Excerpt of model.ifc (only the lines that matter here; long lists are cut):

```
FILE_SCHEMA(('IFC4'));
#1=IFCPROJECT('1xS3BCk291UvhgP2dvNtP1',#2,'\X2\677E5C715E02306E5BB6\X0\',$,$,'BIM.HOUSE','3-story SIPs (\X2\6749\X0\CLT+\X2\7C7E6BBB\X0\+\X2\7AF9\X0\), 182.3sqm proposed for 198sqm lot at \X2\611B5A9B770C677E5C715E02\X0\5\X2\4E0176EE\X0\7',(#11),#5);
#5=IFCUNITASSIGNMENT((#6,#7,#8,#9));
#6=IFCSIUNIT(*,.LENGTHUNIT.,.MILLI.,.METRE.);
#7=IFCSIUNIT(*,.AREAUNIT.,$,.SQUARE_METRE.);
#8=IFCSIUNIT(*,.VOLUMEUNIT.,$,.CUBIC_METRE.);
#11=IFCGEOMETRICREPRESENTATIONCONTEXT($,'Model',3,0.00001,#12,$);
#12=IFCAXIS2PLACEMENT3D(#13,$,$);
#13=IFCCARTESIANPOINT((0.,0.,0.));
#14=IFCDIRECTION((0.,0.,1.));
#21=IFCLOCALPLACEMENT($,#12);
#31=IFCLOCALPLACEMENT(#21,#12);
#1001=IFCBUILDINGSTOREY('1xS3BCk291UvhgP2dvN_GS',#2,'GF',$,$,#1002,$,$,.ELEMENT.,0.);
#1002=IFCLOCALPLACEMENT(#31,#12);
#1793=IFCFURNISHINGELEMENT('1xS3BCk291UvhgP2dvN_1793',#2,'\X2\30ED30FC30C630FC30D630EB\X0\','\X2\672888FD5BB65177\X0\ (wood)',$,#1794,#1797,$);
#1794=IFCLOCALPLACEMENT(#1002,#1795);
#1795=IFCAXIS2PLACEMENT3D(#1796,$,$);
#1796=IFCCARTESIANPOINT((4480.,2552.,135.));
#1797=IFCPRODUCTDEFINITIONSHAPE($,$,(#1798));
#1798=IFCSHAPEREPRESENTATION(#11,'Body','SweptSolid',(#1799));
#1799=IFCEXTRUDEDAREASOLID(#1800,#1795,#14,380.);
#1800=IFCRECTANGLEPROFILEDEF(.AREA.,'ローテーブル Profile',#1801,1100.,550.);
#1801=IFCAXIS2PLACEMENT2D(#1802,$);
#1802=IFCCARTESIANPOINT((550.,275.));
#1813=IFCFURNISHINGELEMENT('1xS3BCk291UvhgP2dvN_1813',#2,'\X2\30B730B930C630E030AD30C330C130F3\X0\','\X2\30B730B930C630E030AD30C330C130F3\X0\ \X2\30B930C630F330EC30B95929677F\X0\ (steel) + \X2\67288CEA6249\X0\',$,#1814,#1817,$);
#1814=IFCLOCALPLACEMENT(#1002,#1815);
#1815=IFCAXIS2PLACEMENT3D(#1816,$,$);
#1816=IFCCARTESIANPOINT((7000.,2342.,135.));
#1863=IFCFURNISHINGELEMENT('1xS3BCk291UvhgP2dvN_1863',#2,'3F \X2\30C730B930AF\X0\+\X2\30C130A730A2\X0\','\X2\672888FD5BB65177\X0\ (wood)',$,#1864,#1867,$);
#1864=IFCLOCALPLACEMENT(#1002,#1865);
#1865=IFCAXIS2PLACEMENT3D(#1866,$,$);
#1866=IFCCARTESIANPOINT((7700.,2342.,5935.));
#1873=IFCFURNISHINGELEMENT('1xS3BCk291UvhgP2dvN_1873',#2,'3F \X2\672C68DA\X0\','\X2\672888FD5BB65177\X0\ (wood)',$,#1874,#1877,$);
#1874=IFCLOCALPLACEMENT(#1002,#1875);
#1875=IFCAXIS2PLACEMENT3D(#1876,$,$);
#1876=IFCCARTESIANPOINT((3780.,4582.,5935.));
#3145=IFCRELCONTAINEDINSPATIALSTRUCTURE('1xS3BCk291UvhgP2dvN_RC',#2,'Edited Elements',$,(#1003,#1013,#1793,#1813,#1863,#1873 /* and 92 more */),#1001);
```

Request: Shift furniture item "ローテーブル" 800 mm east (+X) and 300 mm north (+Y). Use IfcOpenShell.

```python
import ifcopenshell
import ifcopenshell.api.geometry
import ifcopenshell.util.placement
import ifcopenshell.util.unit

model = ifcopenshell.open("model.ifc")
unit_scale = ifcopenshell.util.unit.calculate_unit_scale(model)

item = model.by_guid("1xS3BCk291UvhgP2dvN_1793")
matrix = ifcopenshell.util.placement.get_local_placement(item.ObjectPlacement)
matrix[0, 3] += 0.8 / unit_scale
matrix[1, 3] += 0.3 / unit_scale
ifcopenshell.api.geometry.edit_object_placement(model, product=item, matrix=matrix, is_si=False)

print(ifcopenshell.util.placement.get_local_placement(item.ObjectPlacement).round(3) + 0.0)

model.write("model_rev.ifc")
```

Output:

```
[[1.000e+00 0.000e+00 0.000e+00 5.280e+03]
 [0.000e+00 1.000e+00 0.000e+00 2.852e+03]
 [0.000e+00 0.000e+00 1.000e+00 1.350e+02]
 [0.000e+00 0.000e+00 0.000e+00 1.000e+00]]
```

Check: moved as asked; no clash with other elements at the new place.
